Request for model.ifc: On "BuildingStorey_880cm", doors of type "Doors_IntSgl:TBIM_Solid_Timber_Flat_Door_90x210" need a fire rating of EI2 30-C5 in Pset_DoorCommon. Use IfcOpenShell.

First a look at what the model holds.

```python
import ifcopenshell
import ifcopenshell.util.element

model = ifcopenshell.open("model.ifc")
print(model.schema)
storey = next(s for s in model.by_type("IfcBuildingStorey") if s.Name == "BuildingStorey_880cm")
doors = [e for e in ifcopenshell.util.element.get_decomposition(storey) if e.is_a("IfcDoor")]
seen = {}
for e in doors:
    element_type = ifcopenshell.util.element.get_type(e)
    key = (element_type.Name if element_type != e and element_type else None, ifcopenshell.util.element.get_pset(e, "Pset_DoorCommon", "FireRating"))
    seen[key] = seen.get(key, 0) + 1
for (name, value), count in sorted(seen.items(), key=str):
    print(count, "x", name, "|", value)
```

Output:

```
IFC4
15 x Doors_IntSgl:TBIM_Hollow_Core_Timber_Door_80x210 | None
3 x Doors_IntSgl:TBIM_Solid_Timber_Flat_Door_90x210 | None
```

```python
import ifcopenshell
import ifcopenshell.api.pset
import ifcopenshell.util.element

model = ifcopenshell.open("model.ifc")

storey = next(s for s in model.by_type("IfcBuildingStorey") if s.Name == "BuildingStorey_880cm")
doors = [e for e in ifcopenshell.util.element.get_decomposition(storey) if e.is_a("IfcDoor")]

count = 0
for e in doors:
    element_type = ifcopenshell.util.element.get_type(e)
    if element_type in (None, e) or element_type.Name != "Doors_IntSgl:TBIM_Solid_Timber_Flat_Door_90x210":
        continue
    # add_pset returns the element's existing set when there is one.
    pset = ifcopenshell.api.pset.add_pset(model, product=e, name="Pset_DoorCommon")
    ifcopenshell.api.pset.edit_pset(model, pset=pset, properties={"FireRating": "EI2 30-C5"})
    count += 1

print(count, "doors updated")

model.write("model_v2.ifc")
```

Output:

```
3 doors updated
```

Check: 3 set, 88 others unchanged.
